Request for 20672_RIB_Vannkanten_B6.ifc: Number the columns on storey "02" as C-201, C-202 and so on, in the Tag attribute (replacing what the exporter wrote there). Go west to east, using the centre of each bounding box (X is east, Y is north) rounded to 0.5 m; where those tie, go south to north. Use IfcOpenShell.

First a look at what the model holds.

```python
import ifcopenshell
import ifcopenshell.util.element
import ifcopenshell.util.placement

model = ifcopenshell.open("20672_RIB_Vannkanten_B6.ifc")
print(model.schema)
storey = next(s for s in model.by_type("IfcBuildingStorey") if s.Name == "02")
columns = [e for e in ifcopenshell.util.element.get_decomposition(storey) if e.is_a("IfcColumn")]
for e in sorted(columns, key=lambda e: e.id()):
    origin = ifcopenshell.util.placement.get_local_placement(e.ObjectPlacement)[:3, 3]
    print(e.id(), e.Tag, e.Name, origin.round(2) + 0.0, sep=" | ")
```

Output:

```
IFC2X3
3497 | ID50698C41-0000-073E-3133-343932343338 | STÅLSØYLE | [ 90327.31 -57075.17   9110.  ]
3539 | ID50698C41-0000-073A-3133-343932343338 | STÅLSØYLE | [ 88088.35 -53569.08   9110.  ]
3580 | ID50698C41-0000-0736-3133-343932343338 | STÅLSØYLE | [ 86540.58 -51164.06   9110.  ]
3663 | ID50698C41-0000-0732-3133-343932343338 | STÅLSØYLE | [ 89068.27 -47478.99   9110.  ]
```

```python
import ifcopenshell
import ifcopenshell.geom
import ifcopenshell.util.element
import ifcopenshell.util.shape

model = ifcopenshell.open("20672_RIB_Vannkanten_B6.ifc")
settings = ifcopenshell.geom.settings()
settings.set("use-world-coords", True)


def centre(element):
    shape = ifcopenshell.geom.create_shape(settings, element)
    return ifcopenshell.util.shape.get_bbox_centroid(shape.geometry)


storey = next(s for s in model.by_type("IfcBuildingStorey") if s.Name == "02")
columns = [e for e in ifcopenshell.util.element.get_decomposition(storey) if e.is_a("IfcColumn")]

# Insertion points can sit at a corner or the storey origin, so sort by the geometry (in metres).
centres = {e: centre(e) for e in columns}
columns.sort(key=lambda e: (round(centres[e][0] / 0.5), centres[e][1]))

for i, e in enumerate(columns, start=1):
    number = f"C-2{i:02d}"
    e.Tag = number
    print(e.id(), number)

model.write("20672_RIB_Vannkanten_B6_edited.ifc")
```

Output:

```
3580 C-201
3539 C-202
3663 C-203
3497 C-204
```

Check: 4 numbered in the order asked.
